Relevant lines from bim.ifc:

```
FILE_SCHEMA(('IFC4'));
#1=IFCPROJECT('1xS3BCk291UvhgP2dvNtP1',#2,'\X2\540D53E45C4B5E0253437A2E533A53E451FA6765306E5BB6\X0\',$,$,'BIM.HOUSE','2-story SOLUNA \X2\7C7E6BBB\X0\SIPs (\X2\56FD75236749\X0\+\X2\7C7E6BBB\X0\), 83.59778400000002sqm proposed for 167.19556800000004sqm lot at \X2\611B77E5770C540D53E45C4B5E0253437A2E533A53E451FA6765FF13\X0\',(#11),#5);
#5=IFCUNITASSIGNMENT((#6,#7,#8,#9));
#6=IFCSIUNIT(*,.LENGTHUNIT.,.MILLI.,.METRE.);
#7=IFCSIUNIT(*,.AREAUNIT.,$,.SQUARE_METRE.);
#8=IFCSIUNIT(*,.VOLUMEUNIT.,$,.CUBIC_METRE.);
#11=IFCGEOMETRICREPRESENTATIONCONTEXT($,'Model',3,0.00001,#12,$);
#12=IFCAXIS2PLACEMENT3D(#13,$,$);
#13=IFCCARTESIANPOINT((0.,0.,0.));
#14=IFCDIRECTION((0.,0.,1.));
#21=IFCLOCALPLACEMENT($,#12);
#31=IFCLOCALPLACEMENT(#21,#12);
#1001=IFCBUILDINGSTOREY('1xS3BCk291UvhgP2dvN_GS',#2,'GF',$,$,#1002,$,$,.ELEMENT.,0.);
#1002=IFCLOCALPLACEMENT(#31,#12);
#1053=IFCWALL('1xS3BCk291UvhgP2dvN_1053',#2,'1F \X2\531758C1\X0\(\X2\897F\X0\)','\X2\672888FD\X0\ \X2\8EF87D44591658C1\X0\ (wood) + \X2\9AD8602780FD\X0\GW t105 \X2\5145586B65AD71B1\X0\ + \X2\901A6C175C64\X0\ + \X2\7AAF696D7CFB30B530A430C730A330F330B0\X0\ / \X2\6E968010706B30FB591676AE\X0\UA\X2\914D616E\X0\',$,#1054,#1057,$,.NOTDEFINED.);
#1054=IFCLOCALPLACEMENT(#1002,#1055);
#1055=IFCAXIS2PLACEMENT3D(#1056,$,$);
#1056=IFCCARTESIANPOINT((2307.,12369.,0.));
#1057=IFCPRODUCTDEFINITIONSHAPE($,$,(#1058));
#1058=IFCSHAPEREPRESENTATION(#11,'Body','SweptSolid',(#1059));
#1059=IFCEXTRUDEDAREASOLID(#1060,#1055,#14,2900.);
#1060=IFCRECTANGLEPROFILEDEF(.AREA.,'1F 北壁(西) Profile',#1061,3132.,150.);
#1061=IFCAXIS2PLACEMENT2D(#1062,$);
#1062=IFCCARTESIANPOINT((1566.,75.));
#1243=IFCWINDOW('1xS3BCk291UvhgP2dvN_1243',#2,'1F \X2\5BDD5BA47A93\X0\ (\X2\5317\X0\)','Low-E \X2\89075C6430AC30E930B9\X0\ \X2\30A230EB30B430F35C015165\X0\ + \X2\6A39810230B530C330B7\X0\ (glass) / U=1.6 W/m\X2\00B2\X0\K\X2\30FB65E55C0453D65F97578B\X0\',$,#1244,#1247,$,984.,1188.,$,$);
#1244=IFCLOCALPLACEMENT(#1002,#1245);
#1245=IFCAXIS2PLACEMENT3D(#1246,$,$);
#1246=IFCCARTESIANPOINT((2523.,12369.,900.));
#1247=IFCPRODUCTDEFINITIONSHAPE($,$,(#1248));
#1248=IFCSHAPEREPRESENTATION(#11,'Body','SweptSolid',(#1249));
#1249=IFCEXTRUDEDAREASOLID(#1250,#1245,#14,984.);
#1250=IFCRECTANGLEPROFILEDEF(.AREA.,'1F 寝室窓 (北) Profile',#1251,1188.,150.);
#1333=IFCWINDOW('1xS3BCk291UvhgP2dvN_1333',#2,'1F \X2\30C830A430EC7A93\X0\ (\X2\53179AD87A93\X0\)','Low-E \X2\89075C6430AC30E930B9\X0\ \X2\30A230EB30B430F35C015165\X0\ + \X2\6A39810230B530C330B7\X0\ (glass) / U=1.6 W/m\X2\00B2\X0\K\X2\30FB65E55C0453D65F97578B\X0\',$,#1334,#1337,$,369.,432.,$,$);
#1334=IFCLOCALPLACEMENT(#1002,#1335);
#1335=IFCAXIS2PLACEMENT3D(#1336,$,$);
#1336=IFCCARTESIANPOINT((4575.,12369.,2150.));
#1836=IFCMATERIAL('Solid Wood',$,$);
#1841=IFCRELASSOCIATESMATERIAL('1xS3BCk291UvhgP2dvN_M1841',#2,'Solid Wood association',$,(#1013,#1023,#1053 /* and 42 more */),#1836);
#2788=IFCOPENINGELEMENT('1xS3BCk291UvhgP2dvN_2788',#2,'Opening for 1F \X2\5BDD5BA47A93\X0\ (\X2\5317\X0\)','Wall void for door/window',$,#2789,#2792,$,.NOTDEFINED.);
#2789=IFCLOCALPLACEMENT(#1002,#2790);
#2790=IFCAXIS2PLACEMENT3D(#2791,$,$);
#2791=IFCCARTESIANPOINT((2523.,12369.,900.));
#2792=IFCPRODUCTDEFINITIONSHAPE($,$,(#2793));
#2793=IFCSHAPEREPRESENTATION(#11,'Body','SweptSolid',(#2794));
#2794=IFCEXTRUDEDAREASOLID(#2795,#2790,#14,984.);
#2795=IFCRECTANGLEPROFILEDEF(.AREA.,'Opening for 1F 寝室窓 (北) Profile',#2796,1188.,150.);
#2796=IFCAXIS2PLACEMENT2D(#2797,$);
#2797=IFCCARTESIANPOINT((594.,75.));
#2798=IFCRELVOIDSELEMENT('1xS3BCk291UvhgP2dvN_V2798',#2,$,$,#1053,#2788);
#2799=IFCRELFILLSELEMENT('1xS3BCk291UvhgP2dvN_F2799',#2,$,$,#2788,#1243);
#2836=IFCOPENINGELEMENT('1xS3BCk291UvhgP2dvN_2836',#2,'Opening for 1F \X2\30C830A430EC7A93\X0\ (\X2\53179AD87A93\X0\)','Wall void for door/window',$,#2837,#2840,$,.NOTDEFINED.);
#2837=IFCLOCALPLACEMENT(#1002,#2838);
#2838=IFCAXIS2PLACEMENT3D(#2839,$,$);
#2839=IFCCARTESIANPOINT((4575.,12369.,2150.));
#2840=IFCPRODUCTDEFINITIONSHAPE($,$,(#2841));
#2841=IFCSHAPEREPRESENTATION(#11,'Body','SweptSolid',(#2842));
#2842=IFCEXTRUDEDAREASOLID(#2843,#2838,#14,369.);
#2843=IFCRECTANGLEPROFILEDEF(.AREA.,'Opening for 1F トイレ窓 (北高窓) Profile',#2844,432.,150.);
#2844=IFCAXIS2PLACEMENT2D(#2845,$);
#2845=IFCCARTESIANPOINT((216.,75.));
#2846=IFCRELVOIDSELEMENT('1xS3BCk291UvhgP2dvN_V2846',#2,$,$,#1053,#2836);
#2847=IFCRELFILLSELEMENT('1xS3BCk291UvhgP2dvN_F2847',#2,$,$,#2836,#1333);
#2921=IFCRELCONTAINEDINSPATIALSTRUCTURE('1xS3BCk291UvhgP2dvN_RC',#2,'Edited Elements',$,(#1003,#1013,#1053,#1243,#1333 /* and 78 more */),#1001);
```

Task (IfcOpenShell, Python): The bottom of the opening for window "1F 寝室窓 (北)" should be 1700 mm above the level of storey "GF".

```python
import numpy as np
import ifcopenshell
import ifcopenshell.api.geometry
import ifcopenshell.geom
import ifcopenshell.util.element
import ifcopenshell.util.placement
import ifcopenshell.util.shape
import ifcopenshell.util.unit

model = ifcopenshell.open("bim.ifc")
unit_scale = ifcopenshell.util.unit.calculate_unit_scale(model)

window = model.by_id(1243)
opening = window.FillsVoids[0].RelatingOpeningElement
storey = ifcopenshell.util.element.get_container(window, ifc_class="IfcBuildingStorey")
level = ifcopenshell.util.placement.get_local_placement(storey.ObjectPlacement)[2, 3]

# The opening's origin need not be at the sill, so measure its lowest point.
shape = ifcopenshell.geom.create_shape(ifcopenshell.geom.settings(), opening)
bottom = ifcopenshell.util.shape.get_shape_bottom_elevation(shape, shape.geometry) / unit_scale
dz = level + 1.7 / unit_scale - bottom

shift = np.array([0.0, 0.0, dz])
# The window is not placed relative to its opening, so move both.
for product in (opening, window):
    matrix = ifcopenshell.util.placement.get_local_placement(product.ObjectPlacement)
    matrix[:3, 3] += shift
    ifcopenshell.api.geometry.edit_object_placement(model, product=product, matrix=matrix, is_si=False)

print(f"moved by {dz * unit_scale:+.3f} m")

model.write("bim_updated.ifc")
```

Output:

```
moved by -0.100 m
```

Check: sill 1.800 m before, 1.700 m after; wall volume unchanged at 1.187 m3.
